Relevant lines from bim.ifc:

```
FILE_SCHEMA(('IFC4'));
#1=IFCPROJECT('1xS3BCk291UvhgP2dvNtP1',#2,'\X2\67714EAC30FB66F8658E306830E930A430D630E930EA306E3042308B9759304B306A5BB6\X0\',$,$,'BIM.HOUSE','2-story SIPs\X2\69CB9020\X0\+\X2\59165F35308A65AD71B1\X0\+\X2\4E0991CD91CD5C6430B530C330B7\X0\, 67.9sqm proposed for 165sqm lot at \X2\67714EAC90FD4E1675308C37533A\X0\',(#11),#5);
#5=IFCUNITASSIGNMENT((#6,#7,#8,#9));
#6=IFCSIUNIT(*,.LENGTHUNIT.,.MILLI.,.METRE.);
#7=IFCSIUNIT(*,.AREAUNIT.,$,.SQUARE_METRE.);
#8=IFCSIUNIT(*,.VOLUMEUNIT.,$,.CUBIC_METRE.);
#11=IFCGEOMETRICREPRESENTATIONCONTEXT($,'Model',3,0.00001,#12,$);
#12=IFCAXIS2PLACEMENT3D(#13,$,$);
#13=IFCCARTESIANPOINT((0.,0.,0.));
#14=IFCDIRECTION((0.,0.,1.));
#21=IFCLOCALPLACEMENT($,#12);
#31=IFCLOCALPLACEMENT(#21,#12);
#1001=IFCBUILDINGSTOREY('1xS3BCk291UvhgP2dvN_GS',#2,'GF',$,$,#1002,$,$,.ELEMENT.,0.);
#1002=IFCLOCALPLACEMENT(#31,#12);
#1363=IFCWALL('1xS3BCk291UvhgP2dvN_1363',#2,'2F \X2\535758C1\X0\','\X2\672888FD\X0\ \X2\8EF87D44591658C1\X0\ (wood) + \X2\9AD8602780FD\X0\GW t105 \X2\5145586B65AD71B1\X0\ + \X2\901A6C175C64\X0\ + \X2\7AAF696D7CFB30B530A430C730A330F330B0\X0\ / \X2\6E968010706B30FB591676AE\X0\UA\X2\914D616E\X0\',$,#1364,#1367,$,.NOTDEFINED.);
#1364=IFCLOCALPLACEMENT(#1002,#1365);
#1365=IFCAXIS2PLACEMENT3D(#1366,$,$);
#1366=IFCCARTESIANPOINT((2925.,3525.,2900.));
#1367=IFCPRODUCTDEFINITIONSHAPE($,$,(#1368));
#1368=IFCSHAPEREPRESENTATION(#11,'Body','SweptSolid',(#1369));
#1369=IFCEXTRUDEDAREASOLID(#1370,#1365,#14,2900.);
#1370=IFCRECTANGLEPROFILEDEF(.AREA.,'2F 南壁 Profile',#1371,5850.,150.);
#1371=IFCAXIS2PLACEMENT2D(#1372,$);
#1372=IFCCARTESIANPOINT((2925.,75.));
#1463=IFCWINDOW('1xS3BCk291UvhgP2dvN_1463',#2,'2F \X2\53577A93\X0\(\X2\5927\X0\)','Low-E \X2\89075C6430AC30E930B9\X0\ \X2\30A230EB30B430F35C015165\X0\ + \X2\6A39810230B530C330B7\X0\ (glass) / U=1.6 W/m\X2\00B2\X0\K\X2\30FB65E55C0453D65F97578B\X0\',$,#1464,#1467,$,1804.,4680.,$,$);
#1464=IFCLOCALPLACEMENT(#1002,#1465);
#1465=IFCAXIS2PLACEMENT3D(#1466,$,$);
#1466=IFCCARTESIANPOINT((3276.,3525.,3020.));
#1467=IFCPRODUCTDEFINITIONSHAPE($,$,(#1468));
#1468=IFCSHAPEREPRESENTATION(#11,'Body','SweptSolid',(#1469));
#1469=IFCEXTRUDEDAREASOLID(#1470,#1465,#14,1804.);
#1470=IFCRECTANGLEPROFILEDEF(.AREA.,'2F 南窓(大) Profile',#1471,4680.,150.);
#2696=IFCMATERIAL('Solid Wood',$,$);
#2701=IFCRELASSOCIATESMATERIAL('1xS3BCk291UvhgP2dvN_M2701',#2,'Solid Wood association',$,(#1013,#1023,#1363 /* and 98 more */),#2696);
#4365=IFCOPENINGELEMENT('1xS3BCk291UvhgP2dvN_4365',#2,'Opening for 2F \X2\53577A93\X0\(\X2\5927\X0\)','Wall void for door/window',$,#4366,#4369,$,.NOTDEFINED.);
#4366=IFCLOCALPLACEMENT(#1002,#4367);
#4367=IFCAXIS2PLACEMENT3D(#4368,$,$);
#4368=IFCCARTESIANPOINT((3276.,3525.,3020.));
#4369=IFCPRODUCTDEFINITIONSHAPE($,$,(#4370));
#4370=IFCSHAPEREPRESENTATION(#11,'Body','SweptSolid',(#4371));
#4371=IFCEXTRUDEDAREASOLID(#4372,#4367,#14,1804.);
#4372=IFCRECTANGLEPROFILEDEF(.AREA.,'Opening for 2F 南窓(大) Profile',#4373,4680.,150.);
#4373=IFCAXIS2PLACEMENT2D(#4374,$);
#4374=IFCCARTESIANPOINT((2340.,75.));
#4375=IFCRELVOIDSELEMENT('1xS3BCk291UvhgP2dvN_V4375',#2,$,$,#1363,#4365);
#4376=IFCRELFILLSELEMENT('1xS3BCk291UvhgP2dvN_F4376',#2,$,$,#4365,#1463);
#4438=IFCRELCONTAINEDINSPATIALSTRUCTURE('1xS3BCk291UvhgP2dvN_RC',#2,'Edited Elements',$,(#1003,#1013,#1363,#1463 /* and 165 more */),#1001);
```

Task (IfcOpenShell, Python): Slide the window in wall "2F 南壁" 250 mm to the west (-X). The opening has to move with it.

```python
import ifcopenshell
import ifcopenshell.api.geometry
import ifcopenshell.util.placement
import ifcopenshell.util.unit

model = ifcopenshell.open("bim.ifc")
unit_scale = ifcopenshell.util.unit.calculate_unit_scale(model)

window = model.by_guid("1xS3BCk291UvhgP2dvN_1463")
opening = window.FillsVoids[0].RelatingOpeningElement
wall = opening.VoidsElements[0].RelatingBuildingElement

wall_matrix = ifcopenshell.util.placement.get_local_placement(wall.ObjectPlacement)
shift = wall_matrix[:3, 0] * -0.25 / unit_scale
before = ifcopenshell.util.placement.get_local_placement(window.ObjectPlacement)[:3, 3].copy()

# The window is not placed relative to its opening, so move both.
for product in (opening, window):
    matrix = ifcopenshell.util.placement.get_local_placement(product.ObjectPlacement)
    matrix[:3, 3] += shift
    ifcopenshell.api.geometry.edit_object_placement(model, product=product, matrix=matrix, is_si=False)

after = ifcopenshell.util.placement.get_local_placement(window.ObjectPlacement)[:3, 3]
print("window moved by", (after - before).round(3) + 0.0)

model.write("bim-out.ifc")
```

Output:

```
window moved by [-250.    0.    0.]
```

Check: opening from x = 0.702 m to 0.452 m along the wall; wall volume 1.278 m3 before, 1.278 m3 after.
